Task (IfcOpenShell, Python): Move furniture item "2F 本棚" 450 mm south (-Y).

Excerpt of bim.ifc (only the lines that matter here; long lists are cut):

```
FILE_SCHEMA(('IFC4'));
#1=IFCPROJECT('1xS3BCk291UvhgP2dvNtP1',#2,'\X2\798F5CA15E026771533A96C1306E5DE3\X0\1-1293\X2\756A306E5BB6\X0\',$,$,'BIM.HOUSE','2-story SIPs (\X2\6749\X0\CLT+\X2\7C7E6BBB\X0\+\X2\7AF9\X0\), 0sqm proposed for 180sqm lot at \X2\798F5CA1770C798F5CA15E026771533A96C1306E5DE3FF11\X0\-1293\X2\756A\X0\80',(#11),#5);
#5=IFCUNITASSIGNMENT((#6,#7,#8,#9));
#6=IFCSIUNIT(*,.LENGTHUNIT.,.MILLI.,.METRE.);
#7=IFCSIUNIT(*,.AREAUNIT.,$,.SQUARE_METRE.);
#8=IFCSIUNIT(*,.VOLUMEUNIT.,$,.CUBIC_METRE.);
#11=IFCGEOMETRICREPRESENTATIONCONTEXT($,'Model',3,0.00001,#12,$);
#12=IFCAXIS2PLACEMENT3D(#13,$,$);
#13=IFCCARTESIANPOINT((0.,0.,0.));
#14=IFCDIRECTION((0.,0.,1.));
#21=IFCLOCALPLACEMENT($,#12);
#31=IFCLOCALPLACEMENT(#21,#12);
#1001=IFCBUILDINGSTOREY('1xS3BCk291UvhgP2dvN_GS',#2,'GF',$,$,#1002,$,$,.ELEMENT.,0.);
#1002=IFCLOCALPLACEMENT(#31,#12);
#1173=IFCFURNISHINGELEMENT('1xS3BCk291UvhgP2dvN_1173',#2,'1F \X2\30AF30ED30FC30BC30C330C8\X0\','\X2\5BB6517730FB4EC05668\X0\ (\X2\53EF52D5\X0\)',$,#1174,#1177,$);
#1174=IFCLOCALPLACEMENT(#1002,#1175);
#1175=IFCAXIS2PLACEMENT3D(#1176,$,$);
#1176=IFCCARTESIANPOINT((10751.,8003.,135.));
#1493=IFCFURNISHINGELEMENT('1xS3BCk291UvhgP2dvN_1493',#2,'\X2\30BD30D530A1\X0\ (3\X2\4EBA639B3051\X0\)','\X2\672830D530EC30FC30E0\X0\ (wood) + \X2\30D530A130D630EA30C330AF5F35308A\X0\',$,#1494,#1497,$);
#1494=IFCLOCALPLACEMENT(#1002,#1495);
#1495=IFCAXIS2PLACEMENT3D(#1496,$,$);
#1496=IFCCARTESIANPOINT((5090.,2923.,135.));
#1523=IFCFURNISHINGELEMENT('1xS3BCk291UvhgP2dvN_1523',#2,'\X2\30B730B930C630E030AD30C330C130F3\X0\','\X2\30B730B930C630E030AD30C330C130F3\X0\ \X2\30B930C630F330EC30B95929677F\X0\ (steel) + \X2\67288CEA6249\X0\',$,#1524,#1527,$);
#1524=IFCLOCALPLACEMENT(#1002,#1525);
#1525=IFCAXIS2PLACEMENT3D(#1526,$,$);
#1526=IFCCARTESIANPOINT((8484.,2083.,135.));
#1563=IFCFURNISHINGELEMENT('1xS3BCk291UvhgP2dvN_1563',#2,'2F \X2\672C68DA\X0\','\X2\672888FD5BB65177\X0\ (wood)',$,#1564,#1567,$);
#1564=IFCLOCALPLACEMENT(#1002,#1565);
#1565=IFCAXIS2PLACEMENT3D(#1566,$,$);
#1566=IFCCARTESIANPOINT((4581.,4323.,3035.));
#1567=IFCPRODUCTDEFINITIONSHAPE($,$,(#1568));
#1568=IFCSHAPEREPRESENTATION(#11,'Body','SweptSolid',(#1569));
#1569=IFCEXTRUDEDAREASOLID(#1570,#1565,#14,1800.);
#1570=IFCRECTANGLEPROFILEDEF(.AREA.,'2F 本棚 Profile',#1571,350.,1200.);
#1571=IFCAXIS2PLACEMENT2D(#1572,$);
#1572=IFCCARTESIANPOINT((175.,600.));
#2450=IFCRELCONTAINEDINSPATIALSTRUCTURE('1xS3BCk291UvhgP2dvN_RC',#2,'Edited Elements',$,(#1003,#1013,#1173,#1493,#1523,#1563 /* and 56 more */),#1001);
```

```python
import ifcopenshell
import ifcopenshell.api.geometry
import ifcopenshell.util.placement

model = ifcopenshell.open("bim.ifc")

item = model.by_guid("1xS3BCk291UvhgP2dvN_1563")
matrix = ifcopenshell.util.placement.get_local_placement(item.ObjectPlacement)
matrix[1, 3] -= 450.0
ifcopenshell.api.geometry.edit_object_placement(model, product=item, matrix=matrix, is_si=False)

print(ifcopenshell.util.placement.get_local_placement(item.ObjectPlacement).round(3) + 0.0)

model.write("bim_updated.ifc")
```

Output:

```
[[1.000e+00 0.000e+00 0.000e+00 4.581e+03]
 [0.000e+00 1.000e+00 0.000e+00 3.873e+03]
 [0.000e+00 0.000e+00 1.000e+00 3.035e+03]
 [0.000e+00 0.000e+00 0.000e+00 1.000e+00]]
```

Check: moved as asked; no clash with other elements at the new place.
